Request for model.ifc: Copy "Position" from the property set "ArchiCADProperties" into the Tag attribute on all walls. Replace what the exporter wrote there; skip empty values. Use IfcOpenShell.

First a look at what the model holds.

```python
import ifcopenshell
import ifcopenshell.util.element

model = ifcopenshell.open("model.ifc")
print(model.schema)
walls = model.by_type("IfcWall")
print(len(walls), "walls")
for e in walls[:8]:
    source = ifcopenshell.util.element.get_pset(e, "ArchiCADProperties", "Position")
    target = e.Tag
    print(e.id(), repr(source), repr(target), sep=" | ")
```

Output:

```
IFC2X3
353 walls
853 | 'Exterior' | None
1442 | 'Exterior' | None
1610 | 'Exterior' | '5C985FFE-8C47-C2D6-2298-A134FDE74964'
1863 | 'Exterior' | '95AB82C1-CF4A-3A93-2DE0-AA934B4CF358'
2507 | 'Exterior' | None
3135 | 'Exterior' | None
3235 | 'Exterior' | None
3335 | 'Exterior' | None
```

```python
import ifcopenshell
import ifcopenshell.util.element

model = ifcopenshell.open("model.ifc")

count = 0
for e in model.by_type("IfcWall"):
    value = ifcopenshell.util.element.get_pset(e, "ArchiCADProperties", "Position")
    current = e.Tag
    if not value or not value.strip() or current == value:
        continue
    e.Tag = value
    count += 1

print(count, "walls updated")

model.write("model_updated.ifc")
```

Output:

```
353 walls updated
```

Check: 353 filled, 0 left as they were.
